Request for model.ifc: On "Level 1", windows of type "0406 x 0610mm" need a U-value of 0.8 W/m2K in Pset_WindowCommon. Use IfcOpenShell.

First a look at what the model holds.

```python
import ifcopenshell
import ifcopenshell.util.element

model = ifcopenshell.open("model.ifc")
print(model.schema)
storey = next(s for s in model.by_type("IfcBuildingStorey") if s.Name == "Level 1")
windows = [e for e in ifcopenshell.util.element.get_decomposition(storey) if e.is_a("IfcWindow")]
seen = {}
for e in windows:
    element_type = ifcopenshell.util.element.get_type(e)
    key = (element_type.Name if element_type != e and element_type else None, ifcopenshell.util.element.get_pset(e, "Pset_WindowCommon", "ThermalTransmittance"))
    seen[key] = seen.get(key, 0) + 1
for (name, value), count in sorted(seen.items(), key=str):
    print(count, "x", name, "|", value)
```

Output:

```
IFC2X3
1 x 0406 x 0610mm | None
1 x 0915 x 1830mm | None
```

```python
import ifcopenshell
import ifcopenshell.api.pset
import ifcopenshell.util.element

model = ifcopenshell.open("model.ifc")

storey = next(s for s in model.by_type("IfcBuildingStorey") if s.Name == "Level 1")
windows = [e for e in ifcopenshell.util.element.get_decomposition(storey) if e.is_a("IfcWindow")]

count = 0
for e in windows:
    element_type = ifcopenshell.util.element.get_type(e)
    if element_type in (None, e) or element_type.Name != "0406 x 0610mm":
        continue
    # add_pset returns the element's existing set when there is one.
    pset = ifcopenshell.api.pset.add_pset(model, product=e, name="Pset_WindowCommon")
    ifcopenshell.api.pset.edit_pset(model, pset=pset, properties={"ThermalTransmittance": 0.8})
    count += 1

print(count, "windows updated")

model.write("model-out.ifc")
```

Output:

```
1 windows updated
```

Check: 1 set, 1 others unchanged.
